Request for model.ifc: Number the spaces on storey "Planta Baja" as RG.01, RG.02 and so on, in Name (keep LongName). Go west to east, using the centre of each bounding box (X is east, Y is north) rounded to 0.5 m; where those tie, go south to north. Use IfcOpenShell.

First a look at what the model holds.

```python
import ifcopenshell
import ifcopenshell.util.element
import ifcopenshell.util.placement

model = ifcopenshell.open("model.ifc")
print(model.schema)
storey = next(s for s in model.by_type("IfcBuildingStorey") if s.Name == "Planta Baja")
spaces = [e for e in ifcopenshell.util.element.get_decomposition(storey) if e.is_a("IfcSpace")]
for e in sorted(spaces, key=lambda e: e.id()):
    origin = ifcopenshell.util.placement.get_local_placement(e.ObjectPlacement)[:3, 3]
    print(e.id(), e.Name, e.LongName, origin.round(2) + 0.0, sep=" | ")
```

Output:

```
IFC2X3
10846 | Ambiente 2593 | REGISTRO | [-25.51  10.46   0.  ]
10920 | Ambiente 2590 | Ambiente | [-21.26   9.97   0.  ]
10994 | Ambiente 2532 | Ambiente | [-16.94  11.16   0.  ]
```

```python
import ifcopenshell
import ifcopenshell.geom
import ifcopenshell.util.element
import ifcopenshell.util.shape

model = ifcopenshell.open("model.ifc")
settings = ifcopenshell.geom.settings()
settings.set("use-world-coords", True)


def centre(element):
    shape = ifcopenshell.geom.create_shape(settings, element)
    return ifcopenshell.util.shape.get_bbox_centroid(shape.geometry)


storey = next(s for s in model.by_type("IfcBuildingStorey") if s.Name == "Planta Baja")
spaces = [e for e in ifcopenshell.util.element.get_decomposition(storey) if e.is_a("IfcSpace")]

# Insertion points can sit at a corner or the storey origin, so sort by the geometry (in metres).
centres = {e: centre(e) for e in spaces}
spaces.sort(key=lambda e: (round(centres[e][0] / 0.5), centres[e][1]))

for i, e in enumerate(spaces, start=1):
    number = f"RG.{i:02d}"
    e.Name = number
    print(e.id(), number)

model.write("model_v2.ifc")
```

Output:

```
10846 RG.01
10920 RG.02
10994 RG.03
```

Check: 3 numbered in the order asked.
